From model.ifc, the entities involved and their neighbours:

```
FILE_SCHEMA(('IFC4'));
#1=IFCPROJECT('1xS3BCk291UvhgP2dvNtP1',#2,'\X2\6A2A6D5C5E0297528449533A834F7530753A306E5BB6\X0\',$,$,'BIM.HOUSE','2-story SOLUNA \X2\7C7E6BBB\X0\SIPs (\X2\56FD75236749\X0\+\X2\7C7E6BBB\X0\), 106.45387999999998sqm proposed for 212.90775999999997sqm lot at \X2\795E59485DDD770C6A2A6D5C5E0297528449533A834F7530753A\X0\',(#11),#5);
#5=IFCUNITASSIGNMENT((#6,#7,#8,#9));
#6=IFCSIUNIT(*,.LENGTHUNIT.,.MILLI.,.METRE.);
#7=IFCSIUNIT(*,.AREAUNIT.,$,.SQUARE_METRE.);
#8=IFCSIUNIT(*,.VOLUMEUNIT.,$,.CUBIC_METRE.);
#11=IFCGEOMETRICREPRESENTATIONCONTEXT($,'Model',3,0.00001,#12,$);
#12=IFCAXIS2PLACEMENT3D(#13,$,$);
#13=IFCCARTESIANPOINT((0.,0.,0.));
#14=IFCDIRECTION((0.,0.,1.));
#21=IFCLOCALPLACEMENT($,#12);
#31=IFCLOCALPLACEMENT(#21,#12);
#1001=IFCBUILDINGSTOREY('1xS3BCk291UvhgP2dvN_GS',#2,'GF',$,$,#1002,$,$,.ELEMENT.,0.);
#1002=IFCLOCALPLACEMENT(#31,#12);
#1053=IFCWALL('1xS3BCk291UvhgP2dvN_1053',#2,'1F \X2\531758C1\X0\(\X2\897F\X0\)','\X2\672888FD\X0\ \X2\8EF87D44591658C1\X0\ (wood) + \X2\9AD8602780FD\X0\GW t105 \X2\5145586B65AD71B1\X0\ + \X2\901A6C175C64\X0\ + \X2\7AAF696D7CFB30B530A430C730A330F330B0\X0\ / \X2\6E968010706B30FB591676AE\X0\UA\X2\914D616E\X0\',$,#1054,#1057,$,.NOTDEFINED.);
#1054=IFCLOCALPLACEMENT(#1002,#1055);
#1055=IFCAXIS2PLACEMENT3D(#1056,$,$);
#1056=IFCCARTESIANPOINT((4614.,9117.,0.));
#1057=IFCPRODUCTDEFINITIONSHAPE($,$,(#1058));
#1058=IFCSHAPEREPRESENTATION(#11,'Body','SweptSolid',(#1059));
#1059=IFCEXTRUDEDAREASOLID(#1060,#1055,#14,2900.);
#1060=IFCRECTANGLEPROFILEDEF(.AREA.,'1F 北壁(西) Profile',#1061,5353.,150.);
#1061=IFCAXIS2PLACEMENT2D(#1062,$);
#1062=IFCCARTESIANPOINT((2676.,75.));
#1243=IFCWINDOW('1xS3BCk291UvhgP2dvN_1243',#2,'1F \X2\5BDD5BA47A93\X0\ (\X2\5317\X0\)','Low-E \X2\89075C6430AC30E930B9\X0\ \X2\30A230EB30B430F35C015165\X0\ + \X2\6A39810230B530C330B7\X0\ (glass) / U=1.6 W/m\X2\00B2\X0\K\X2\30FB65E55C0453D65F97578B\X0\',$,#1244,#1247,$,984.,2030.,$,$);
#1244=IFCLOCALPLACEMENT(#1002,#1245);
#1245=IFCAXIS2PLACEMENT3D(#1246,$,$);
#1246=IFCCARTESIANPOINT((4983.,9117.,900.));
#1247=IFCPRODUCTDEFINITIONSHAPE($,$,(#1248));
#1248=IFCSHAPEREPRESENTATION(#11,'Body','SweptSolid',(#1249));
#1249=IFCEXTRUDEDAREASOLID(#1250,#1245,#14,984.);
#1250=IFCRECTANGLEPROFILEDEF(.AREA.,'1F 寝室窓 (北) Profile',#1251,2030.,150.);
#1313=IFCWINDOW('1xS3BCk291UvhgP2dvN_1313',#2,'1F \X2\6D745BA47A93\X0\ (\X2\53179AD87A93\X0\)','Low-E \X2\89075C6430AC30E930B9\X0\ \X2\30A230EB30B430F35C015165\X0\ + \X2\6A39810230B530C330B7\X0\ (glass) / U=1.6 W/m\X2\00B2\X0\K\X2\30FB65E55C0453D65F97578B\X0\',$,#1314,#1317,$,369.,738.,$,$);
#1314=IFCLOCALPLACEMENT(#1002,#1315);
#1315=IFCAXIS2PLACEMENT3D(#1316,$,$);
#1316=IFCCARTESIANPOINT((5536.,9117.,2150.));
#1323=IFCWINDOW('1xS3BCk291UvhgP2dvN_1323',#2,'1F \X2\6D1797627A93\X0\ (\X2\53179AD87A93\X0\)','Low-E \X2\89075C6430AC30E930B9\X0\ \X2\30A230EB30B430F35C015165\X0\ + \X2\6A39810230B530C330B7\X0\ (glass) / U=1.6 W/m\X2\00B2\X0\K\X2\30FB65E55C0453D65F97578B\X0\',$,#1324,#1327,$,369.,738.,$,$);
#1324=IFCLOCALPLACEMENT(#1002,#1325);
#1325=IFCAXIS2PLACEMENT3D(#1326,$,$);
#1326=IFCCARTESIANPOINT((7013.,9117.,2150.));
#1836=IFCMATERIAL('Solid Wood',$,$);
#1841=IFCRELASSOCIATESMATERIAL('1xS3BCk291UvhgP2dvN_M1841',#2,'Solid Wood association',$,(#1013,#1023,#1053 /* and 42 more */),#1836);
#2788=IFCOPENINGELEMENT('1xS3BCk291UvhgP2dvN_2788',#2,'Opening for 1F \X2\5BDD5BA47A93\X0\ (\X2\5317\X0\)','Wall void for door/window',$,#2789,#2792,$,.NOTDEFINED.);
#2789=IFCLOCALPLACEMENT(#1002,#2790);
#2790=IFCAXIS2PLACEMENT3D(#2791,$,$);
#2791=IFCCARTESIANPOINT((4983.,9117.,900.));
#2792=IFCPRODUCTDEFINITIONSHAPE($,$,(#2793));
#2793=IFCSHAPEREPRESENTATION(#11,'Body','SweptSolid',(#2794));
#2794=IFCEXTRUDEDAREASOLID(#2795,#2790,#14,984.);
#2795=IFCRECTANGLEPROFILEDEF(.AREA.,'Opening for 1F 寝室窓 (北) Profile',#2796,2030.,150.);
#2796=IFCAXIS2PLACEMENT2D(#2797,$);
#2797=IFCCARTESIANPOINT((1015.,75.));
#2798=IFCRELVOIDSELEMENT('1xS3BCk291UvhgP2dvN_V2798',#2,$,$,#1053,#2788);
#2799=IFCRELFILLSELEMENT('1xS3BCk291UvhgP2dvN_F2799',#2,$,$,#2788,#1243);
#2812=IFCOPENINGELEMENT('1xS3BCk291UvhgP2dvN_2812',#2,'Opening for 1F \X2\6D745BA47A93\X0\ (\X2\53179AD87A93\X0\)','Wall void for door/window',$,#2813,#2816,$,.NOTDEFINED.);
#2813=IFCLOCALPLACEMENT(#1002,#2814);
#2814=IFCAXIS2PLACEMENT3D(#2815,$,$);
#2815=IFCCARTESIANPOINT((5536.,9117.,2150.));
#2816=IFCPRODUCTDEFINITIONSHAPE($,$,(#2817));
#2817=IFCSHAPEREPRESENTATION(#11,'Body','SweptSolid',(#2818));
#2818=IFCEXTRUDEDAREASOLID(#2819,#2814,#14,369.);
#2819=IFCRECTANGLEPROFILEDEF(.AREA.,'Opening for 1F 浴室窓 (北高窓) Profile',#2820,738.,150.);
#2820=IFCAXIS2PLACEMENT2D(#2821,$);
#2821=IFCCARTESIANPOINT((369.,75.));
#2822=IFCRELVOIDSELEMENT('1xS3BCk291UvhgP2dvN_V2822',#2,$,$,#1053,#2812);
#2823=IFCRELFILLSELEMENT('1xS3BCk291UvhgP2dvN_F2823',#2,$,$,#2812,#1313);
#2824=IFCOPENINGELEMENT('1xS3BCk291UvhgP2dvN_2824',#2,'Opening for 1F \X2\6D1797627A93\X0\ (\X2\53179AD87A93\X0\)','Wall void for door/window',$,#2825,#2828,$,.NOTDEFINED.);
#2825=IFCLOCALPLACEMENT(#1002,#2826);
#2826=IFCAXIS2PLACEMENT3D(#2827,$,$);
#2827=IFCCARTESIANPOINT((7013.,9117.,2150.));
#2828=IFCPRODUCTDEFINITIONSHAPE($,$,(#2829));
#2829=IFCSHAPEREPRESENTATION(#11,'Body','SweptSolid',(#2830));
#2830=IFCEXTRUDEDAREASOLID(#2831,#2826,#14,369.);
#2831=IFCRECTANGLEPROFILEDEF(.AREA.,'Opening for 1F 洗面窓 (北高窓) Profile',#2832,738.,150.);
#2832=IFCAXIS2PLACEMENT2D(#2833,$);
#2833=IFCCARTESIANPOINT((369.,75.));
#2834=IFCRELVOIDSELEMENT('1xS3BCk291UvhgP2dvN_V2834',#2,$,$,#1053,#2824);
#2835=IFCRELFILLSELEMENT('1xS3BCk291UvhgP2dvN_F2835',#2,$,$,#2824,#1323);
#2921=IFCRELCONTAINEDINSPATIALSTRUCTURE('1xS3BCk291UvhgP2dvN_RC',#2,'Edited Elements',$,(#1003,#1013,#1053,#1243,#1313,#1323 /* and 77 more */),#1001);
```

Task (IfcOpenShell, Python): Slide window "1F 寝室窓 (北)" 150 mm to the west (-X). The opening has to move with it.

```python
import ifcopenshell
import ifcopenshell.api.geometry
import ifcopenshell.util.placement

model = ifcopenshell.open("model.ifc")

window = model.by_guid("1xS3BCk291UvhgP2dvN_1243")
opening = window.FillsVoids[0].RelatingOpeningElement
wall = opening.VoidsElements[0].RelatingBuildingElement

wall_matrix = ifcopenshell.util.placement.get_local_placement(wall.ObjectPlacement)
shift = wall_matrix[:3, 0] * -150.0
before = ifcopenshell.util.placement.get_local_placement(window.ObjectPlacement)[:3, 3].copy()

# The window is not placed relative to its opening, so move both.
for product in (opening, window):
    matrix = ifcopenshell.util.placement.get_local_placement(product.ObjectPlacement)
    matrix[:3, 3] += shift
    ifcopenshell.api.geometry.edit_object_placement(model, product=product, matrix=matrix, is_si=False)

after = ifcopenshell.util.placement.get_local_placement(window.ObjectPlacement)[:3, 3]
print("window moved by", (after - before).round(3) + 0.0)

model.write("model_edited.ifc")
```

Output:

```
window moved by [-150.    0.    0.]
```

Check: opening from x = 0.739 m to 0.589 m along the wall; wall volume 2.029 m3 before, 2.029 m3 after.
